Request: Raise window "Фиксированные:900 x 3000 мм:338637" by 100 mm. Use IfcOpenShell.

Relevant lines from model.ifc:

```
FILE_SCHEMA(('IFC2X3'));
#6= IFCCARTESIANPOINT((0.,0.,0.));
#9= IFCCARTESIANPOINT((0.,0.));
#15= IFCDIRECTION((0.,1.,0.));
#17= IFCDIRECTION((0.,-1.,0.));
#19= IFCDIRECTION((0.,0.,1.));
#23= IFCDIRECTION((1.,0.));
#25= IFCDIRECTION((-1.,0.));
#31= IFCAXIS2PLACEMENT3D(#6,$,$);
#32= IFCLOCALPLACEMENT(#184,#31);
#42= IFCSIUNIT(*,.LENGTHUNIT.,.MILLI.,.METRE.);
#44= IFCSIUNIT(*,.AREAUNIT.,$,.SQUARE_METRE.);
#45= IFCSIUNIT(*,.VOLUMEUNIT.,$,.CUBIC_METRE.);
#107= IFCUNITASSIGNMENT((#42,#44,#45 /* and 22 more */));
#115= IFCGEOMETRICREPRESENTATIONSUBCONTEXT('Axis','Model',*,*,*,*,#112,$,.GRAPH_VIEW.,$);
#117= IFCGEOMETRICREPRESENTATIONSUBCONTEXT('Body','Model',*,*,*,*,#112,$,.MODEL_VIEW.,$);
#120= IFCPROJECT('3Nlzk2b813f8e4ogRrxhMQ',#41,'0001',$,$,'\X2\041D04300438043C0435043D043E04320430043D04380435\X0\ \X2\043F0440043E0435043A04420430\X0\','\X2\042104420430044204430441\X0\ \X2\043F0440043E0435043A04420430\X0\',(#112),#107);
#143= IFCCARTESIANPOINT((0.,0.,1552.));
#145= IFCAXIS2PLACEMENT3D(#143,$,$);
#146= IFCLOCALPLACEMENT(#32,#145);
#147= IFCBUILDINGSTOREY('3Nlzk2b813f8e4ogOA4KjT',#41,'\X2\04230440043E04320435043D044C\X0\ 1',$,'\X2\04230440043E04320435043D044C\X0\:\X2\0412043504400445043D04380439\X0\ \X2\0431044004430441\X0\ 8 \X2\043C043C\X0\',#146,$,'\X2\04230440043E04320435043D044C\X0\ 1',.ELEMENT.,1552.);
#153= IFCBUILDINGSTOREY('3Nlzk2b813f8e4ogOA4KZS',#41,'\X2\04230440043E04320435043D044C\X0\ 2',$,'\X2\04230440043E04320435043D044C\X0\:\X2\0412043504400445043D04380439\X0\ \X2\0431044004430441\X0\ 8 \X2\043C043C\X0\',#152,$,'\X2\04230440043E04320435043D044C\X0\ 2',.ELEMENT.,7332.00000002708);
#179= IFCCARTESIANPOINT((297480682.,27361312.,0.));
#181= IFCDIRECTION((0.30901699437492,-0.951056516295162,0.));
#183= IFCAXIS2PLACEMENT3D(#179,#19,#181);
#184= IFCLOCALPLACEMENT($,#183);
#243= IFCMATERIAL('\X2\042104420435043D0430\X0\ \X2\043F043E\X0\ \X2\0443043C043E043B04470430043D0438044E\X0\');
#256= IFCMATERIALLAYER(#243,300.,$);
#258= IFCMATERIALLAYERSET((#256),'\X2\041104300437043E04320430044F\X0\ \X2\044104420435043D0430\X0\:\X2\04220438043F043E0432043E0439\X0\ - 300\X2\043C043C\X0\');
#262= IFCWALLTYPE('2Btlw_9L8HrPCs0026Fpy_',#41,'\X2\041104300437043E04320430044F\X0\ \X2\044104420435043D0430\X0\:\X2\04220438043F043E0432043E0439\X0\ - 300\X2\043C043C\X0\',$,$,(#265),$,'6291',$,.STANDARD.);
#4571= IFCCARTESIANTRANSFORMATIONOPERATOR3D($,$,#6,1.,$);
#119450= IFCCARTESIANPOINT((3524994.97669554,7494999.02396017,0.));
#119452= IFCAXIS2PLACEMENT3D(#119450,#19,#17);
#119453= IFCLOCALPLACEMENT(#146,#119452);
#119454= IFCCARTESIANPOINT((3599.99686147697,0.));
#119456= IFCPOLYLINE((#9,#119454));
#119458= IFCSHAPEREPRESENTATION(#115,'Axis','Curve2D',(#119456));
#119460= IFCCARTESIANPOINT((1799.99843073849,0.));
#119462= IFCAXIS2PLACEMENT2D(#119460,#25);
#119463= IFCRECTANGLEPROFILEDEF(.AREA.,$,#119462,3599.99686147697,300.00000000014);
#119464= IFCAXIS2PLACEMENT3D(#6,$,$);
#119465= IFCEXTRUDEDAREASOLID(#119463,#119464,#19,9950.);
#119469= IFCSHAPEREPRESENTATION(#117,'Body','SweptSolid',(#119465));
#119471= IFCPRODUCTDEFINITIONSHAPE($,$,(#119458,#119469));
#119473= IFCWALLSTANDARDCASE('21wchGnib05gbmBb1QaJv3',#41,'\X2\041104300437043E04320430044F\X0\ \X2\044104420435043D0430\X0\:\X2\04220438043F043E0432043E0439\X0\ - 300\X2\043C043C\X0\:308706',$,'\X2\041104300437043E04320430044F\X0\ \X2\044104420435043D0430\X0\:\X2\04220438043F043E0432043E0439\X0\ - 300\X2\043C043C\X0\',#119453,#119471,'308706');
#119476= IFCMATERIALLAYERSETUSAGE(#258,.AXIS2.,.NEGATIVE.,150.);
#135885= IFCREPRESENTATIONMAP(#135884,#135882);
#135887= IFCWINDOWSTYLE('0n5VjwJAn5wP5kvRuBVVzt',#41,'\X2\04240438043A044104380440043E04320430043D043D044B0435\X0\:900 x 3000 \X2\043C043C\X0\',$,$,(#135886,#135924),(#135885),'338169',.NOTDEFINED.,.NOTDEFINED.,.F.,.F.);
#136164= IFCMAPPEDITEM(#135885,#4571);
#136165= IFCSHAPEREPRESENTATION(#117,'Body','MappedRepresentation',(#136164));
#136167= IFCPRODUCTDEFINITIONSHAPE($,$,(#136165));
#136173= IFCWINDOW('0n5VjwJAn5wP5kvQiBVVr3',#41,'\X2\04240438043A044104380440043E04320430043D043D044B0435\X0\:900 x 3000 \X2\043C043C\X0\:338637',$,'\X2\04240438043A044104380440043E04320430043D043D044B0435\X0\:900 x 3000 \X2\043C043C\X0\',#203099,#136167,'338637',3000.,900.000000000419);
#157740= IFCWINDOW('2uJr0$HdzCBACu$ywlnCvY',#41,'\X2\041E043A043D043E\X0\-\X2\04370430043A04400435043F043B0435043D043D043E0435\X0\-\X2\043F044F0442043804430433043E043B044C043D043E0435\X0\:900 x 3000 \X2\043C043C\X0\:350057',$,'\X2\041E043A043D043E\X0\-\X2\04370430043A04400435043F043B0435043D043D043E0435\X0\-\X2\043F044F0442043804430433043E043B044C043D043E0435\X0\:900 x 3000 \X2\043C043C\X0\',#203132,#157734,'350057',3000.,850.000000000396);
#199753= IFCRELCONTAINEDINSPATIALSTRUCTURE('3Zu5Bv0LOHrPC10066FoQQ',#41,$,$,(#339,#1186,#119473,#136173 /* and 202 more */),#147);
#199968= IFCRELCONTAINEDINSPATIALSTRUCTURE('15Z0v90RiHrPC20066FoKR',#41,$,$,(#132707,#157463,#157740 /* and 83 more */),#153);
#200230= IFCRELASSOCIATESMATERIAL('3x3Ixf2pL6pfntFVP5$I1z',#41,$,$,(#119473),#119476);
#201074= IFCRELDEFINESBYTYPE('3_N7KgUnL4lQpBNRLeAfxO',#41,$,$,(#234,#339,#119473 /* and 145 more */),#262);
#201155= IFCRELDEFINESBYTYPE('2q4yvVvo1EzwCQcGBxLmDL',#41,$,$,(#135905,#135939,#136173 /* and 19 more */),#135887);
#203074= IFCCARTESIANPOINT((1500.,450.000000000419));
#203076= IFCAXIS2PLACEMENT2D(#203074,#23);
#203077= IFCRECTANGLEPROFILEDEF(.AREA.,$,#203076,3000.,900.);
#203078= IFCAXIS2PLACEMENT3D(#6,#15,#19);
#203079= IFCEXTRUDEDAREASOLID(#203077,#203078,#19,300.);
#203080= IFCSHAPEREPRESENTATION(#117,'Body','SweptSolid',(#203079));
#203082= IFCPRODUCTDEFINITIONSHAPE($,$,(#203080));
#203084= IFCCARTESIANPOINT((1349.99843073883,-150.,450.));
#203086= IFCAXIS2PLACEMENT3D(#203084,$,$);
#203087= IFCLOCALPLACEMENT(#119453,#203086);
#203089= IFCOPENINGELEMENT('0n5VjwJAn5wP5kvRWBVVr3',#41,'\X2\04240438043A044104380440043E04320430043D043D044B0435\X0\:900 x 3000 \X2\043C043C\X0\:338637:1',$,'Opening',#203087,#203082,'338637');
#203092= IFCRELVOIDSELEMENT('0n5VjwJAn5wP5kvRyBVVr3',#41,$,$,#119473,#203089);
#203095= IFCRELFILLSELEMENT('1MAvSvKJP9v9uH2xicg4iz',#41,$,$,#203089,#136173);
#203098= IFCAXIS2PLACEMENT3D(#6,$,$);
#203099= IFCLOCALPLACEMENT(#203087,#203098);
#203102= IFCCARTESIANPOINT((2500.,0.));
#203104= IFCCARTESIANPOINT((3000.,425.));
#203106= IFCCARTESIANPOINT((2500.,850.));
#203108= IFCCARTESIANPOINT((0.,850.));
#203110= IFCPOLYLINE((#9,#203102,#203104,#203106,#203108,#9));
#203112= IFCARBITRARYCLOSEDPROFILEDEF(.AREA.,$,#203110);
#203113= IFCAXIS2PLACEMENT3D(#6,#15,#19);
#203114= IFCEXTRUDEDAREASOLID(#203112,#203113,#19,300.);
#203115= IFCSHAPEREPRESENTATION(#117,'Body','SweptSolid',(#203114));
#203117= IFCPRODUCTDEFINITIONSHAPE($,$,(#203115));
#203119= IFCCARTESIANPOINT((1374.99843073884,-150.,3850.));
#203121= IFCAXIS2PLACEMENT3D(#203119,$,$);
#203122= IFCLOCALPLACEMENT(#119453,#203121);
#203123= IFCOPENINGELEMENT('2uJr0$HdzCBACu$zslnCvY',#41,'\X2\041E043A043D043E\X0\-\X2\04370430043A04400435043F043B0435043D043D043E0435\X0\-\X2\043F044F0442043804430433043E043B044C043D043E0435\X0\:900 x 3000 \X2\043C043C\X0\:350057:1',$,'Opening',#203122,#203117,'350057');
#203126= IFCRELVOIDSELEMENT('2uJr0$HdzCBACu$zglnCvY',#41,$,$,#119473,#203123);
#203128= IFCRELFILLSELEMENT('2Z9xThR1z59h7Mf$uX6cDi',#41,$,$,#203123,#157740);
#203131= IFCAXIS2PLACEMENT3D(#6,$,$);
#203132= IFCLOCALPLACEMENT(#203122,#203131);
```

```python
import numpy as np
import ifcopenshell
import ifcopenshell.api.geometry
import ifcopenshell.util.placement
import ifcopenshell.util.unit

model = ifcopenshell.open("model.ifc")
unit_scale = ifcopenshell.util.unit.calculate_unit_scale(model)

window = model.by_guid("0n5VjwJAn5wP5kvQiBVVr3")
opening = window.FillsVoids[0].RelatingOpeningElement
dz = 0.1 / unit_scale

shift = np.array([0.0, 0.0, dz])
# The window is placed relative to its opening, so it follows when the opening moves.
matrix = ifcopenshell.util.placement.get_local_placement(opening.ObjectPlacement)
matrix[:3, 3] += shift
ifcopenshell.api.geometry.edit_object_placement(
    model, product=opening, matrix=matrix, is_si=False, should_transform_children=True
)

print(f"moved by {dz * unit_scale:+.3f} m")

model.write("model_updated.ifc")
```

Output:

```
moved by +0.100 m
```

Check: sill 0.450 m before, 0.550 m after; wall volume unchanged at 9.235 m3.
